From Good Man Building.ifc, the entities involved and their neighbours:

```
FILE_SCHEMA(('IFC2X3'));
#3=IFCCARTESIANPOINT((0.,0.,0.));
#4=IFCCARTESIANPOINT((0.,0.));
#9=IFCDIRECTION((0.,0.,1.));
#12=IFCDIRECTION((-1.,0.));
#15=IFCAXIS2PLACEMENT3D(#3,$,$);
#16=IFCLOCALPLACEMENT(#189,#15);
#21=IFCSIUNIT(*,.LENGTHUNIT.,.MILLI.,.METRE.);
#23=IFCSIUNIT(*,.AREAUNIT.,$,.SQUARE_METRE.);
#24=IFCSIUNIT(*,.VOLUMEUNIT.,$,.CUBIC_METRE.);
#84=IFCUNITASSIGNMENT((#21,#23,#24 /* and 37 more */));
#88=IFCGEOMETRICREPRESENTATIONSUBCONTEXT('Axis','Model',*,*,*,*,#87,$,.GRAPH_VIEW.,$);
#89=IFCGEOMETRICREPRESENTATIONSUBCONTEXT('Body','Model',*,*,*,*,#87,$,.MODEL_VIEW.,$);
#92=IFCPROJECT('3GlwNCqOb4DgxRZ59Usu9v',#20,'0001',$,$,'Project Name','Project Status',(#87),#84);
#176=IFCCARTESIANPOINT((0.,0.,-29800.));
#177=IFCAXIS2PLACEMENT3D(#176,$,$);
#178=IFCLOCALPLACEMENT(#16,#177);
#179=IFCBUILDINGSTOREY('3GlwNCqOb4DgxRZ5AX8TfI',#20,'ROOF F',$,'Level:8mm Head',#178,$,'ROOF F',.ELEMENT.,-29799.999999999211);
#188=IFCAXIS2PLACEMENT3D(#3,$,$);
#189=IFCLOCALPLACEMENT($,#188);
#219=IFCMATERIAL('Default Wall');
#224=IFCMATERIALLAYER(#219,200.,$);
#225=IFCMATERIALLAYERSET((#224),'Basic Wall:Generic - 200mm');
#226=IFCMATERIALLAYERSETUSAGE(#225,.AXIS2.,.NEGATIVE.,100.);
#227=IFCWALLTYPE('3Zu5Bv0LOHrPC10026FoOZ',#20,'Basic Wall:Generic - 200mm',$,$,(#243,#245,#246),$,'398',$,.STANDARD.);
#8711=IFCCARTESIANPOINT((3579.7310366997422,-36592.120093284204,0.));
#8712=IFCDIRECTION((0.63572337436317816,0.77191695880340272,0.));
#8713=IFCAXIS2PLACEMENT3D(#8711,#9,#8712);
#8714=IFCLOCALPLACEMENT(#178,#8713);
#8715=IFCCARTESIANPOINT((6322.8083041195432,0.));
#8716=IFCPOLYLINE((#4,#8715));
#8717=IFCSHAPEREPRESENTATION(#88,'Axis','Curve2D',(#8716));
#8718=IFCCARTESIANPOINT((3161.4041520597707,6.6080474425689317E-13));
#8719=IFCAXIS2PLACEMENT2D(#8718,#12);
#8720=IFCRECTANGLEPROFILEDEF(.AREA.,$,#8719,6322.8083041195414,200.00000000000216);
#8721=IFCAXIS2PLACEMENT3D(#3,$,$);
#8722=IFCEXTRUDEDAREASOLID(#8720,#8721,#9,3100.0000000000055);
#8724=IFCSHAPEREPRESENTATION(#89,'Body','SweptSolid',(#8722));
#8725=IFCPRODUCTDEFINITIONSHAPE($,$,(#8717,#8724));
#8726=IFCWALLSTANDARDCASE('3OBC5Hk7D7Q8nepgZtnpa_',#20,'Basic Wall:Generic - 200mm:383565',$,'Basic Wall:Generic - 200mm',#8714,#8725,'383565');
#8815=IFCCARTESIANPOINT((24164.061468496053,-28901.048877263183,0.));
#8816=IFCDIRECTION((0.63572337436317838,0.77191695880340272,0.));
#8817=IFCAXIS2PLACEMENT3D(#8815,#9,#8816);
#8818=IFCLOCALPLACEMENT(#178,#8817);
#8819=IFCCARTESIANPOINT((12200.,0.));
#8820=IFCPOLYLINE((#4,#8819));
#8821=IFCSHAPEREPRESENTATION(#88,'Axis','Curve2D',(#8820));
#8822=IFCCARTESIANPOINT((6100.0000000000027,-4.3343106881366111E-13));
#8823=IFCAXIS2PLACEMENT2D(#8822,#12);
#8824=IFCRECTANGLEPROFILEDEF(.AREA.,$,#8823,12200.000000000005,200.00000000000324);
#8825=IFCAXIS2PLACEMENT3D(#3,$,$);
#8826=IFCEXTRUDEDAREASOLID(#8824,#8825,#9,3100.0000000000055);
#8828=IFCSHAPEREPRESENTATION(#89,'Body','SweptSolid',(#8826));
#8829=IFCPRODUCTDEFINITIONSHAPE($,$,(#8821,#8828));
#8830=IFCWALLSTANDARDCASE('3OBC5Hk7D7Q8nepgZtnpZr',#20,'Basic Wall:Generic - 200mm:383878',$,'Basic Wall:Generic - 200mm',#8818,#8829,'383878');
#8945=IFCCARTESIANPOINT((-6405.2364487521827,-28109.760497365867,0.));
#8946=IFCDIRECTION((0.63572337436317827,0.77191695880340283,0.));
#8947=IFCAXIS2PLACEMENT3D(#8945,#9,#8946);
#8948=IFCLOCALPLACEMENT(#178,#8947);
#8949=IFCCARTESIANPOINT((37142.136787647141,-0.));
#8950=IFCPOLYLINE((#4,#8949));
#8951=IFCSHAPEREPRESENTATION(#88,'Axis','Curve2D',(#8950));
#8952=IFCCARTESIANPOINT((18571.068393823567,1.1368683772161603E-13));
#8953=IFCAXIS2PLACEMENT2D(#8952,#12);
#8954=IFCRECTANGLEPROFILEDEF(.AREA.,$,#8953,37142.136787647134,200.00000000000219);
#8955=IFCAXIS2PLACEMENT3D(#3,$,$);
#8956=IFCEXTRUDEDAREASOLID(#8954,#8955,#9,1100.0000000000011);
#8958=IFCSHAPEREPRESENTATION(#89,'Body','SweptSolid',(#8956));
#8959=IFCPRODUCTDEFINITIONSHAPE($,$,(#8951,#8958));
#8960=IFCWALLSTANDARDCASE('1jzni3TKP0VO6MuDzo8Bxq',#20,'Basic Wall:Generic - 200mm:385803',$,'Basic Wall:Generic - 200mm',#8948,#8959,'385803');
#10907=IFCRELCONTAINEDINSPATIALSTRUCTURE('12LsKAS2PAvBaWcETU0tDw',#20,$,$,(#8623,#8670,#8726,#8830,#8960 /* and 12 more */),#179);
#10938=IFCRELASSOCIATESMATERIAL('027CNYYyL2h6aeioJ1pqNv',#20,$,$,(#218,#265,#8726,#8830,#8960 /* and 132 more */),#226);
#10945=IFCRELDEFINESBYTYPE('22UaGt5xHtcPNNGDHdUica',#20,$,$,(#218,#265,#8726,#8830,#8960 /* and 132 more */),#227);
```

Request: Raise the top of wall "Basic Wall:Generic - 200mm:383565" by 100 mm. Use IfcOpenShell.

```python
import ifcopenshell
import ifcopenshell.geom
import ifcopenshell.util.representation
import ifcopenshell.util.shape
import ifcopenshell.util.unit

model = ifcopenshell.open("Good Man Building.ifc")
unit_scale = ifcopenshell.util.unit.calculate_unit_scale(model)
settings = ifcopenshell.geom.settings()


def volume(element):
    """Net volume in cubic metres, openings subtracted."""
    shape = ifcopenshell.geom.create_shape(settings, element)
    return ifcopenshell.util.shape.get_volume(shape.geometry)


wall = model.by_guid("3OBC5Hk7D7Q8nepgZtnpa_")
before = volume(wall)

body = ifcopenshell.util.representation.get_representation(wall, "Model", "Body")
solid = body.Items[0]
old_height = solid.Depth
solid.Depth += 0.1 / unit_scale
after = volume(wall)

print(f"height {old_height:g} -> {solid.Depth:g}, volume {before:.3f} -> {after:.3f} m3")

model.write("Good Man Building_updated.ifc")
```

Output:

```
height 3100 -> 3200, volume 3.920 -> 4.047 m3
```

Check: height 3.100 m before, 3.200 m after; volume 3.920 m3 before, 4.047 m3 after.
